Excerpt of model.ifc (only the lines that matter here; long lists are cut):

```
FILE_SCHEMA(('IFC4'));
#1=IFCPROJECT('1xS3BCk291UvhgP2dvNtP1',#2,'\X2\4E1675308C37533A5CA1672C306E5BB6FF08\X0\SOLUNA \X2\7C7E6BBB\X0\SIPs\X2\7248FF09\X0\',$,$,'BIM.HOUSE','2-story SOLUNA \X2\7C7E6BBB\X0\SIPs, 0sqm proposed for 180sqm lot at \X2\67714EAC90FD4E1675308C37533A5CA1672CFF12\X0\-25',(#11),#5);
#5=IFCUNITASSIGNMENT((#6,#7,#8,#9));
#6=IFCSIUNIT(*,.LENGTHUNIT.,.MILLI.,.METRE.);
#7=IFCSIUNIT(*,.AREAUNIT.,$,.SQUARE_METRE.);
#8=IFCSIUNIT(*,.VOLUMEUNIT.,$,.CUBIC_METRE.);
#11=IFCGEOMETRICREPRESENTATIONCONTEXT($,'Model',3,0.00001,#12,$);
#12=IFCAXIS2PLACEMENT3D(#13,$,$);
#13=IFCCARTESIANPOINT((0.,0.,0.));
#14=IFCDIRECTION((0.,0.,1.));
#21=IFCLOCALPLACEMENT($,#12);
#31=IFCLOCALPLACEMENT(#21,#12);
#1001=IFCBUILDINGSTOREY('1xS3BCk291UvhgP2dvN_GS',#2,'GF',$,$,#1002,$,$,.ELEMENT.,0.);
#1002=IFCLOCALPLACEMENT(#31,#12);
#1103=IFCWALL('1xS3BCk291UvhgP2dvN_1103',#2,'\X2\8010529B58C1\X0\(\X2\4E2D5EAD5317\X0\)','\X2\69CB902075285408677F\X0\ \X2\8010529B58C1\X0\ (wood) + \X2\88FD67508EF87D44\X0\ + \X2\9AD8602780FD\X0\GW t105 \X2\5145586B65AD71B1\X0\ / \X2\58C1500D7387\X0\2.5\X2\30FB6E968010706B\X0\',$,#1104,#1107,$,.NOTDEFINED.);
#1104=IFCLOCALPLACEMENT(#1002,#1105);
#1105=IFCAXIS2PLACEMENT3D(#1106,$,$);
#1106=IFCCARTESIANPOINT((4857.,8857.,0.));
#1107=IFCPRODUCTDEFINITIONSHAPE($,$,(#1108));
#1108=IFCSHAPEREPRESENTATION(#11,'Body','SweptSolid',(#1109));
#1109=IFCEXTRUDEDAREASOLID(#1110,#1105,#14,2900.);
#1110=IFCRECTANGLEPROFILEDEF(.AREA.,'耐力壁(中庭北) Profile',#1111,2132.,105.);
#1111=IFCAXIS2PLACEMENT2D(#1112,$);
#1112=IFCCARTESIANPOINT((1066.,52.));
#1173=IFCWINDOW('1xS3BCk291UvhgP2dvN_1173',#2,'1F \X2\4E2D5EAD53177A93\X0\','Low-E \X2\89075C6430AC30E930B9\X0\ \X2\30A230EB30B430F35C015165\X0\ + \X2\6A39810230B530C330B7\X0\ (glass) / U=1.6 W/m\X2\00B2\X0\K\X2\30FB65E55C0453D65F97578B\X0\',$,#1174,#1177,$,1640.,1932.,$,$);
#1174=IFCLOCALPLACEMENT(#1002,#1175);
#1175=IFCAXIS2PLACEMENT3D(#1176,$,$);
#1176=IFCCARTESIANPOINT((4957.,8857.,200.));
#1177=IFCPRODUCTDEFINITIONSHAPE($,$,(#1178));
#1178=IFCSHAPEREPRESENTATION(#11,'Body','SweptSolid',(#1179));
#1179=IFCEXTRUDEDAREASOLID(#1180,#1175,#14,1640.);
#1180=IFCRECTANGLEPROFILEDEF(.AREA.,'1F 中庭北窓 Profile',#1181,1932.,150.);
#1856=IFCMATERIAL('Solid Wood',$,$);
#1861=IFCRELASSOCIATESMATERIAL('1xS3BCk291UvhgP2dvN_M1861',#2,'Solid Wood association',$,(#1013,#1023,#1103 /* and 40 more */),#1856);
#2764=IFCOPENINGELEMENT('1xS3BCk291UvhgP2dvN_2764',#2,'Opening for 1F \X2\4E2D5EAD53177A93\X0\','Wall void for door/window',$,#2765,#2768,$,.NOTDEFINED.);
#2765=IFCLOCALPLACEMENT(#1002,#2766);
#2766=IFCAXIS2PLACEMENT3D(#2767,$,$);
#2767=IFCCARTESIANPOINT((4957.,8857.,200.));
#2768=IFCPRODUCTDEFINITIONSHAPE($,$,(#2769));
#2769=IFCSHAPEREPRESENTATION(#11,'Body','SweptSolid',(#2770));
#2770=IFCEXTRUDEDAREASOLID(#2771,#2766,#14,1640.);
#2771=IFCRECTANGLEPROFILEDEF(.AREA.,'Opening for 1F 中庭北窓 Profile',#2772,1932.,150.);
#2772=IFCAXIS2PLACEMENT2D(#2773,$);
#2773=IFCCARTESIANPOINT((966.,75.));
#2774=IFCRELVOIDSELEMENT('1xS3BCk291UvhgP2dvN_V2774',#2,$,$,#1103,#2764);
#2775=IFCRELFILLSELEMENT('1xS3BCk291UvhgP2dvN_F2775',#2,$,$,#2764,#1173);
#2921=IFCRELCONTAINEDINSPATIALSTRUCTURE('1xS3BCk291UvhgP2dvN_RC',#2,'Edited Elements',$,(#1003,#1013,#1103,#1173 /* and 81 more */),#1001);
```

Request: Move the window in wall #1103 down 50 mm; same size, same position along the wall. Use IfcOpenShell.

```python
import numpy as np
import ifcopenshell
import ifcopenshell.api.geometry
import ifcopenshell.util.placement
import ifcopenshell.util.unit

model = ifcopenshell.open("model.ifc")
unit_scale = ifcopenshell.util.unit.calculate_unit_scale(model)

window = model.by_id(1173)
opening = window.FillsVoids[0].RelatingOpeningElement
dz = -0.05 / unit_scale

shift = np.array([0.0, 0.0, dz])
# The window is not placed relative to its opening, so move both.
for product in (opening, window):
    matrix = ifcopenshell.util.placement.get_local_placement(product.ObjectPlacement)
    matrix[:3, 3] += shift
    ifcopenshell.api.geometry.edit_object_placement(model, product=product, matrix=matrix, is_si=False)

print(f"moved by {dz * unit_scale:+.3f} m")

model.write("model_updated.ifc")
```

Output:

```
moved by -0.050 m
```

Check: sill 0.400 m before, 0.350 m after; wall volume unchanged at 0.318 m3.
